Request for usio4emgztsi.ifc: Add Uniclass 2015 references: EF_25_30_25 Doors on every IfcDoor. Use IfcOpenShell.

First a look at what the model holds.

```python
import ifcopenshell

model = ifcopenshell.open("usio4emgztsi.ifc")
print(model.schema)
print("classifications:", [c.Name for c in model.by_type("IfcClassification")])
for ifc_class in ("IfcDoor", "IfcRoof", "IfcStair", "IfcWall", "IfcWindow"):
    print(ifc_class, len(model.by_type(ifc_class)))
```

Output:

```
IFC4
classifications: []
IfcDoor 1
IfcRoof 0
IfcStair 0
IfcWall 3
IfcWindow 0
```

```python
import ifcopenshell
import ifcopenshell.api.classification

model = ifcopenshell.open("usio4emgztsi.ifc")

system = ifcopenshell.api.classification.add_classification(model, classification="Uniclass 2015")

codes = {
    "IfcDoor": ("EF_25_30_25", "Doors"),
}
for ifc_class, (code, name) in codes.items():
    products = model.by_type(ifc_class)
    ifcopenshell.api.classification.add_reference(
        model, products=products, classification=system, identification=code, name=name
    )
    print(code, len(products))

model.write("usio4emgztsi_updated.ifc")
```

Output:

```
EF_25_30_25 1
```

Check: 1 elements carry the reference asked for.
